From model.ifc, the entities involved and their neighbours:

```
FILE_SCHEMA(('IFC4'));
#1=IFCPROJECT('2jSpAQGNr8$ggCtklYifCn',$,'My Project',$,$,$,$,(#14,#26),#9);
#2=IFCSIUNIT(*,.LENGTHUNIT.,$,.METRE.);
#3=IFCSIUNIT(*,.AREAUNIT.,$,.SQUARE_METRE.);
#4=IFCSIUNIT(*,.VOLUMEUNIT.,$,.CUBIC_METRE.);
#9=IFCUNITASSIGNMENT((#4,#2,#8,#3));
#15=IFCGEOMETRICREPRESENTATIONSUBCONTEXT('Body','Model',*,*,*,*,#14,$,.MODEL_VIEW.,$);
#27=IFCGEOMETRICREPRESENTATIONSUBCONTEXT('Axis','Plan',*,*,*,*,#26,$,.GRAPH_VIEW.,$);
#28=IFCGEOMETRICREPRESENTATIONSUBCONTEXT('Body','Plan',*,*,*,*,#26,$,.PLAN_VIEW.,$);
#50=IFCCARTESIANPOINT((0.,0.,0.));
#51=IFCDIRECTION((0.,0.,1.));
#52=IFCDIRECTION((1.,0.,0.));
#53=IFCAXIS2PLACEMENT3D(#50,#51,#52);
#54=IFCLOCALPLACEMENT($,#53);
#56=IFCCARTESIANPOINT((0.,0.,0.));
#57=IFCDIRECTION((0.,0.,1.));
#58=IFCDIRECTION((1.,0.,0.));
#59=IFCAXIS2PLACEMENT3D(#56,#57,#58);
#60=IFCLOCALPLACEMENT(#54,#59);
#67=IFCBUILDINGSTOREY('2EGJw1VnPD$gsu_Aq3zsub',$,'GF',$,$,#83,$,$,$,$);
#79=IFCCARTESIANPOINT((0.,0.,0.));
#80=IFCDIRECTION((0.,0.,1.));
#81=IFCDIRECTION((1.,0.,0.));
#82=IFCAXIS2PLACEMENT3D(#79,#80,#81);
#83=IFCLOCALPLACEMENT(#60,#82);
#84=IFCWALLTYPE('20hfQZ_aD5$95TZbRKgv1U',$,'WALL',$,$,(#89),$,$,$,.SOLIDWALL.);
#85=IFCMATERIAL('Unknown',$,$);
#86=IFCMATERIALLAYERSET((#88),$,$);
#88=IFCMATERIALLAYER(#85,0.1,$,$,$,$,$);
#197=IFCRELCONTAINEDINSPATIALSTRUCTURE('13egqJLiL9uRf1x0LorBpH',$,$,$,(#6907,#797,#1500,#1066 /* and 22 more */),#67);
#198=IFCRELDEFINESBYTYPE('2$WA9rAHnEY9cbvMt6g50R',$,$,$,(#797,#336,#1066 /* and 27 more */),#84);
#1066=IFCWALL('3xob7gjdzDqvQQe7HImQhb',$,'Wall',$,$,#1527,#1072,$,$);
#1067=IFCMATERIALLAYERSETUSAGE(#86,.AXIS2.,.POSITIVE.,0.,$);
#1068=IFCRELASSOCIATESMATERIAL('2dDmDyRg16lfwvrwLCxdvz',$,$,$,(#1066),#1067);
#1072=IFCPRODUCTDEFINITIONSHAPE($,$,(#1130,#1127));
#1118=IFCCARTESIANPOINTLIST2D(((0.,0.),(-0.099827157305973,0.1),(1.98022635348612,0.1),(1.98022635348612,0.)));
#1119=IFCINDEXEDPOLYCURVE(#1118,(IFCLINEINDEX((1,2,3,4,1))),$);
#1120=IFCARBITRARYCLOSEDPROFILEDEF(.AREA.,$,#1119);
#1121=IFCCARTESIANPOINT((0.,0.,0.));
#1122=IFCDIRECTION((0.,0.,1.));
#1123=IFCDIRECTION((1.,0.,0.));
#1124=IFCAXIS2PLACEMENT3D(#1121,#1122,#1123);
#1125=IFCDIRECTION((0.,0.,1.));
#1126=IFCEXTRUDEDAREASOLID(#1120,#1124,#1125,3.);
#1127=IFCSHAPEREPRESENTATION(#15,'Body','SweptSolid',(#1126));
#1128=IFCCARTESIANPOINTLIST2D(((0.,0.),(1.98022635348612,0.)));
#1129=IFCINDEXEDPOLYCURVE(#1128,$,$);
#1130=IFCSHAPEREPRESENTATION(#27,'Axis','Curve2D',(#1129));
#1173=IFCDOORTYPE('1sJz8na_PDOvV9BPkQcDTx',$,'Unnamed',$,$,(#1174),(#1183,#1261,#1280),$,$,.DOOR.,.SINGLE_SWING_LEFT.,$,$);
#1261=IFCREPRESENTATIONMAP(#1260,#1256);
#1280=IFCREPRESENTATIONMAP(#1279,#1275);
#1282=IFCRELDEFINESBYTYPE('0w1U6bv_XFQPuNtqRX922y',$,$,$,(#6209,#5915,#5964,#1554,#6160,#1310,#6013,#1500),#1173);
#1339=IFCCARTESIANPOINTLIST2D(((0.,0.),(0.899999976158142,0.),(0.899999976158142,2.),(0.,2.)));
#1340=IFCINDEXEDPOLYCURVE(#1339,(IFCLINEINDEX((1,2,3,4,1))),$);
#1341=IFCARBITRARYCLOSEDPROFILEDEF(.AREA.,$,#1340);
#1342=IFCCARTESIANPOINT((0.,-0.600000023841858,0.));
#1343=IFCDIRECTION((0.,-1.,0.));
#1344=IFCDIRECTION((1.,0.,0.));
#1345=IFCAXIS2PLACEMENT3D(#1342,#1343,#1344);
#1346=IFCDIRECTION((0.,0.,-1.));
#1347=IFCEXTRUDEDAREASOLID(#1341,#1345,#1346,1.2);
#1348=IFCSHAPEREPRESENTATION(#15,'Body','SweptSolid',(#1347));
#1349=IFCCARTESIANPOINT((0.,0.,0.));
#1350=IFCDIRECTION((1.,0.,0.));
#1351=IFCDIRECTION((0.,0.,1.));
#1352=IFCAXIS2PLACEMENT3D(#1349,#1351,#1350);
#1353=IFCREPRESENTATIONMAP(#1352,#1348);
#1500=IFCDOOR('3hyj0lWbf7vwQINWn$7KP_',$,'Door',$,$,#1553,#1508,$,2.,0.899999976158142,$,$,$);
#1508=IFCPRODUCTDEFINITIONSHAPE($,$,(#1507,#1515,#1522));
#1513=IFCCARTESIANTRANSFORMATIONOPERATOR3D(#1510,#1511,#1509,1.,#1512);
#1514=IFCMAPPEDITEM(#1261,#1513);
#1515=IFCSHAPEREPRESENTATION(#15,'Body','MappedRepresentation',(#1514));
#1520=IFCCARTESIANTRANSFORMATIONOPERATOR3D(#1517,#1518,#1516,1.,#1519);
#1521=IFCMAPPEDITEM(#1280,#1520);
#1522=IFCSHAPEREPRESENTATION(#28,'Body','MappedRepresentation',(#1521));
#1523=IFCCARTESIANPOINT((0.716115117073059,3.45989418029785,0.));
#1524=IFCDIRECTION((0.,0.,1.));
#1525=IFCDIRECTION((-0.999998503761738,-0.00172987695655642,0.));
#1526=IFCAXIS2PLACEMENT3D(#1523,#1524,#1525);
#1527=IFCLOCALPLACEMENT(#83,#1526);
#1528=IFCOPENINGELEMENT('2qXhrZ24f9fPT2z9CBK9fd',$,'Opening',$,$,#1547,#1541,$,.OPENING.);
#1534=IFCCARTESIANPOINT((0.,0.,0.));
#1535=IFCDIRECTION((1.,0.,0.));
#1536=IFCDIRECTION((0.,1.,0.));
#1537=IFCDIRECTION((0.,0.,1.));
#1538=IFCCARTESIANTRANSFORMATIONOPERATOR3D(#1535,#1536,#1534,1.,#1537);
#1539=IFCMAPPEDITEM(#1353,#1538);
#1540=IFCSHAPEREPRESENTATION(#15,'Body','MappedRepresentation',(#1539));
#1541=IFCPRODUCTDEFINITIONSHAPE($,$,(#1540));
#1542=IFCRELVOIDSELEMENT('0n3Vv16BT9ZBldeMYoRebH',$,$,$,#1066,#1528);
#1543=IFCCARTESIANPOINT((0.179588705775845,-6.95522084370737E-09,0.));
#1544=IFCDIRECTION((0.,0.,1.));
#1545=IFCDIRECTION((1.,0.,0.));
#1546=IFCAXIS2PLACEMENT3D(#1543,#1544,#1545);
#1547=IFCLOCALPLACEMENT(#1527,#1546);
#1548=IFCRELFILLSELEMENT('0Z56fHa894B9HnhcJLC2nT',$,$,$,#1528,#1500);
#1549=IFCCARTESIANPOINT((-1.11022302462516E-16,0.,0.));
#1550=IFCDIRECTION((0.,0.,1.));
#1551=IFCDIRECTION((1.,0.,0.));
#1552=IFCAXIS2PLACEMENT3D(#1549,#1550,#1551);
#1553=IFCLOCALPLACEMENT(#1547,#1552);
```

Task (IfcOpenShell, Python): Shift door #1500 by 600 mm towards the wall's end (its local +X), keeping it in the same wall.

```python
import ifcopenshell
import ifcopenshell.api.geometry
import ifcopenshell.util.placement
import ifcopenshell.util.unit

model = ifcopenshell.open("model.ifc")
unit_scale = ifcopenshell.util.unit.calculate_unit_scale(model)

door = model.by_id(1500)
opening = door.FillsVoids[0].RelatingOpeningElement
wall = opening.VoidsElements[0].RelatingBuildingElement

wall_matrix = ifcopenshell.util.placement.get_local_placement(wall.ObjectPlacement)
shift = wall_matrix[:3, 0] * 0.6 / unit_scale
before = ifcopenshell.util.placement.get_local_placement(door.ObjectPlacement)[:3, 3].copy()

# The door is placed relative to its opening, so it follows when the opening moves.
matrix = ifcopenshell.util.placement.get_local_placement(opening.ObjectPlacement)
matrix[:3, 3] += shift
ifcopenshell.api.geometry.edit_object_placement(
    model, product=opening, matrix=matrix, is_si=False, should_transform_children=True
)

after = ifcopenshell.util.placement.get_local_placement(door.ObjectPlacement)[:3, 3]
print("door moved by", (after - before).round(3) + 0.0)

model.write("model_edited.ifc")
```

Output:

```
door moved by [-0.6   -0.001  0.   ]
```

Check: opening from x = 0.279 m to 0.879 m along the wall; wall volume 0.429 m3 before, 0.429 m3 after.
